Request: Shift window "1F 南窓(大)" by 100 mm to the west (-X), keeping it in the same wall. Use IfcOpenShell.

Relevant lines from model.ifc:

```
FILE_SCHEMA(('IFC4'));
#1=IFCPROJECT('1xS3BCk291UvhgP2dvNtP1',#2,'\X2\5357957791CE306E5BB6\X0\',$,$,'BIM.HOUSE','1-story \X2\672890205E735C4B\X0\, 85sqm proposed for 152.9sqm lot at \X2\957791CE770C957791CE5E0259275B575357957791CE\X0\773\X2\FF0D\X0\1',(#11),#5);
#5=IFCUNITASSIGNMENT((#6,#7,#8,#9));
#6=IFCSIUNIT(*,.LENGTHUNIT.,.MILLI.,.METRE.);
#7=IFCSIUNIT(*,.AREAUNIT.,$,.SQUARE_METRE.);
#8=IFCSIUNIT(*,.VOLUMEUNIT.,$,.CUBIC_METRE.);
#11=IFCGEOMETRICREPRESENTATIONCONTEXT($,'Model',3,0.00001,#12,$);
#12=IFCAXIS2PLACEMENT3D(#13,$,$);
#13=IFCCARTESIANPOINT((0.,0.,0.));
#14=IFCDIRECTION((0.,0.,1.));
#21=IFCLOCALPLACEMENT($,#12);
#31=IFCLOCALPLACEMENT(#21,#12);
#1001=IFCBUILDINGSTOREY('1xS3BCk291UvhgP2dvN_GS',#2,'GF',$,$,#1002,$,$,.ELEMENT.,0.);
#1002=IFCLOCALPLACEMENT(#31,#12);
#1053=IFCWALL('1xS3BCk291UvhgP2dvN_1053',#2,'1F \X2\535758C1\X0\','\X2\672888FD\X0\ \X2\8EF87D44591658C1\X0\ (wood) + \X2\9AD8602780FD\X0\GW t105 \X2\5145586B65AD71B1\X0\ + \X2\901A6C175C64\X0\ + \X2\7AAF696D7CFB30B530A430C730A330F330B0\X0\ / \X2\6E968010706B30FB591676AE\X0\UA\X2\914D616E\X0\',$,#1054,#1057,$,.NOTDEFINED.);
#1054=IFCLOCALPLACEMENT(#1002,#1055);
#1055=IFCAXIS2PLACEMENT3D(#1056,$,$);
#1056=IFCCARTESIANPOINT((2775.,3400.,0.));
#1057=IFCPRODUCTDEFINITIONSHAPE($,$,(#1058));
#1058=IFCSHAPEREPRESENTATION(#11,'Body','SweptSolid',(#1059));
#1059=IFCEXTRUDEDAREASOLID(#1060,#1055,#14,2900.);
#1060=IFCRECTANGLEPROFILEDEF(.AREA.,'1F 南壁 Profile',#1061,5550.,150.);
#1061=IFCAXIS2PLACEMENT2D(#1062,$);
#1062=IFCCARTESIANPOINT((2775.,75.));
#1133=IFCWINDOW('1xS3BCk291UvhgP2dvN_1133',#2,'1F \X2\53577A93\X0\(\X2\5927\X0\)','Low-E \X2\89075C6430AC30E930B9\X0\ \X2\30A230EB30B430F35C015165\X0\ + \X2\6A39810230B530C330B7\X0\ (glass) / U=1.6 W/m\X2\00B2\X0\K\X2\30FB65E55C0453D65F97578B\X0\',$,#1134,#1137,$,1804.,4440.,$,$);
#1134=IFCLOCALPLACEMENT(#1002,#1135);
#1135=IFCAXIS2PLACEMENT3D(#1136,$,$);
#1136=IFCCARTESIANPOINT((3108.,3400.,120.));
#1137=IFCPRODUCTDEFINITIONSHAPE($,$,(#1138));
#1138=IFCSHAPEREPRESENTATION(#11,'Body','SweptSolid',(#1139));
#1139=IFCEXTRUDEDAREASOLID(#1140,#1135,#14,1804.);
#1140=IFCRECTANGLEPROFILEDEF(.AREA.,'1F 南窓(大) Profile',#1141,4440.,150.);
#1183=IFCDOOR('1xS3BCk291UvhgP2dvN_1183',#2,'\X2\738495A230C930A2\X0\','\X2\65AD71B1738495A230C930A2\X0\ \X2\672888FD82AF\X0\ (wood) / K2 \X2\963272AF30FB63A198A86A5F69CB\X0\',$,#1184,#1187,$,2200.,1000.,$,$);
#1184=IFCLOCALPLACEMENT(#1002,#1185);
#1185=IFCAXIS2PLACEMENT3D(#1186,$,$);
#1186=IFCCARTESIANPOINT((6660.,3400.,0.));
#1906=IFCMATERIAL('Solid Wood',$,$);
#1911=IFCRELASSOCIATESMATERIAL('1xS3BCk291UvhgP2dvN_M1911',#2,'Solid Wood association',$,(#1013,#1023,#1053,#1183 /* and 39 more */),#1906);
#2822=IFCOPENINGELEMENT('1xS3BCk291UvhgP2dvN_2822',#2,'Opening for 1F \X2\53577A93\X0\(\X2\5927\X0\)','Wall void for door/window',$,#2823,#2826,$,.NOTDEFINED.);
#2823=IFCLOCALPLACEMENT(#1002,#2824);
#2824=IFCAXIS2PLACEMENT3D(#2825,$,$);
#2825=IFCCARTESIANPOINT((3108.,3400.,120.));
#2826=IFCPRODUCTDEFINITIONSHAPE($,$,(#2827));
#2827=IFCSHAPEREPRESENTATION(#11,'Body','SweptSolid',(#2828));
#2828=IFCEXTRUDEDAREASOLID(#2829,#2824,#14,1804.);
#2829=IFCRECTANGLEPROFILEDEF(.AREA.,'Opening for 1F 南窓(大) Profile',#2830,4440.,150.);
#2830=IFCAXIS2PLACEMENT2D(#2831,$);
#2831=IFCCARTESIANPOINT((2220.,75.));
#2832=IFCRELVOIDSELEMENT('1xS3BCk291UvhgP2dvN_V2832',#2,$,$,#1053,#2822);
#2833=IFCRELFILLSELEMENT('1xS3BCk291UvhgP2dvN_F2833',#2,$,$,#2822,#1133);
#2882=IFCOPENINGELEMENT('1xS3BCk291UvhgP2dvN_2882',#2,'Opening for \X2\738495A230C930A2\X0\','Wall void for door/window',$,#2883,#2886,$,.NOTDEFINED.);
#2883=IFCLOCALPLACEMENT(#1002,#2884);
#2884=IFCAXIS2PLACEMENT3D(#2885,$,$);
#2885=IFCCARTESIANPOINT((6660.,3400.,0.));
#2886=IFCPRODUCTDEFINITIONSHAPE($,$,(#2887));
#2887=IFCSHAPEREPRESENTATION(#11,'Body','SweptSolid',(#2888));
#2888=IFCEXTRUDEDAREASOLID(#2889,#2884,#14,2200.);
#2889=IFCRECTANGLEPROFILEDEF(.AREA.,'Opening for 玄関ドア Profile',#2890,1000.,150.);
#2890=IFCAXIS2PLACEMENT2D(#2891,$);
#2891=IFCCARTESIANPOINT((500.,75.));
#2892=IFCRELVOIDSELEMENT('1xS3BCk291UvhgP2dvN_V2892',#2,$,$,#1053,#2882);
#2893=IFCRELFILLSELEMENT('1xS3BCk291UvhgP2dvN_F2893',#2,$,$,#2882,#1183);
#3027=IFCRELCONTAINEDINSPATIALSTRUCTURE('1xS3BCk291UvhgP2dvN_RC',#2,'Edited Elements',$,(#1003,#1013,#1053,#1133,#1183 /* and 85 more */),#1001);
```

```python
import ifcopenshell
import ifcopenshell.api.geometry
import ifcopenshell.util.placement
import ifcopenshell.util.unit

model = ifcopenshell.open("model.ifc")
unit_scale = ifcopenshell.util.unit.calculate_unit_scale(model)

window = model.by_guid("1xS3BCk291UvhgP2dvN_1133")
opening = window.FillsVoids[0].RelatingOpeningElement
wall = opening.VoidsElements[0].RelatingBuildingElement

wall_matrix = ifcopenshell.util.placement.get_local_placement(wall.ObjectPlacement)
shift = wall_matrix[:3, 0] * -0.1 / unit_scale
before = ifcopenshell.util.placement.get_local_placement(window.ObjectPlacement)[:3, 3].copy()

# The window is not placed relative to its opening, so move both.
for product in (opening, window):
    matrix = ifcopenshell.util.placement.get_local_placement(product.ObjectPlacement)
    matrix[:3, 3] += shift
    ifcopenshell.api.geometry.edit_object_placement(model, product=product, matrix=matrix, is_si=False)

after = ifcopenshell.util.placement.get_local_placement(window.ObjectPlacement)[:3, 3]
print("window moved by", (after - before).round(3) + 0.0)

model.write("model_updated.ifc")
```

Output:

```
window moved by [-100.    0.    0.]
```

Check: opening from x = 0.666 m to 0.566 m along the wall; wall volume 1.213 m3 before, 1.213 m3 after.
